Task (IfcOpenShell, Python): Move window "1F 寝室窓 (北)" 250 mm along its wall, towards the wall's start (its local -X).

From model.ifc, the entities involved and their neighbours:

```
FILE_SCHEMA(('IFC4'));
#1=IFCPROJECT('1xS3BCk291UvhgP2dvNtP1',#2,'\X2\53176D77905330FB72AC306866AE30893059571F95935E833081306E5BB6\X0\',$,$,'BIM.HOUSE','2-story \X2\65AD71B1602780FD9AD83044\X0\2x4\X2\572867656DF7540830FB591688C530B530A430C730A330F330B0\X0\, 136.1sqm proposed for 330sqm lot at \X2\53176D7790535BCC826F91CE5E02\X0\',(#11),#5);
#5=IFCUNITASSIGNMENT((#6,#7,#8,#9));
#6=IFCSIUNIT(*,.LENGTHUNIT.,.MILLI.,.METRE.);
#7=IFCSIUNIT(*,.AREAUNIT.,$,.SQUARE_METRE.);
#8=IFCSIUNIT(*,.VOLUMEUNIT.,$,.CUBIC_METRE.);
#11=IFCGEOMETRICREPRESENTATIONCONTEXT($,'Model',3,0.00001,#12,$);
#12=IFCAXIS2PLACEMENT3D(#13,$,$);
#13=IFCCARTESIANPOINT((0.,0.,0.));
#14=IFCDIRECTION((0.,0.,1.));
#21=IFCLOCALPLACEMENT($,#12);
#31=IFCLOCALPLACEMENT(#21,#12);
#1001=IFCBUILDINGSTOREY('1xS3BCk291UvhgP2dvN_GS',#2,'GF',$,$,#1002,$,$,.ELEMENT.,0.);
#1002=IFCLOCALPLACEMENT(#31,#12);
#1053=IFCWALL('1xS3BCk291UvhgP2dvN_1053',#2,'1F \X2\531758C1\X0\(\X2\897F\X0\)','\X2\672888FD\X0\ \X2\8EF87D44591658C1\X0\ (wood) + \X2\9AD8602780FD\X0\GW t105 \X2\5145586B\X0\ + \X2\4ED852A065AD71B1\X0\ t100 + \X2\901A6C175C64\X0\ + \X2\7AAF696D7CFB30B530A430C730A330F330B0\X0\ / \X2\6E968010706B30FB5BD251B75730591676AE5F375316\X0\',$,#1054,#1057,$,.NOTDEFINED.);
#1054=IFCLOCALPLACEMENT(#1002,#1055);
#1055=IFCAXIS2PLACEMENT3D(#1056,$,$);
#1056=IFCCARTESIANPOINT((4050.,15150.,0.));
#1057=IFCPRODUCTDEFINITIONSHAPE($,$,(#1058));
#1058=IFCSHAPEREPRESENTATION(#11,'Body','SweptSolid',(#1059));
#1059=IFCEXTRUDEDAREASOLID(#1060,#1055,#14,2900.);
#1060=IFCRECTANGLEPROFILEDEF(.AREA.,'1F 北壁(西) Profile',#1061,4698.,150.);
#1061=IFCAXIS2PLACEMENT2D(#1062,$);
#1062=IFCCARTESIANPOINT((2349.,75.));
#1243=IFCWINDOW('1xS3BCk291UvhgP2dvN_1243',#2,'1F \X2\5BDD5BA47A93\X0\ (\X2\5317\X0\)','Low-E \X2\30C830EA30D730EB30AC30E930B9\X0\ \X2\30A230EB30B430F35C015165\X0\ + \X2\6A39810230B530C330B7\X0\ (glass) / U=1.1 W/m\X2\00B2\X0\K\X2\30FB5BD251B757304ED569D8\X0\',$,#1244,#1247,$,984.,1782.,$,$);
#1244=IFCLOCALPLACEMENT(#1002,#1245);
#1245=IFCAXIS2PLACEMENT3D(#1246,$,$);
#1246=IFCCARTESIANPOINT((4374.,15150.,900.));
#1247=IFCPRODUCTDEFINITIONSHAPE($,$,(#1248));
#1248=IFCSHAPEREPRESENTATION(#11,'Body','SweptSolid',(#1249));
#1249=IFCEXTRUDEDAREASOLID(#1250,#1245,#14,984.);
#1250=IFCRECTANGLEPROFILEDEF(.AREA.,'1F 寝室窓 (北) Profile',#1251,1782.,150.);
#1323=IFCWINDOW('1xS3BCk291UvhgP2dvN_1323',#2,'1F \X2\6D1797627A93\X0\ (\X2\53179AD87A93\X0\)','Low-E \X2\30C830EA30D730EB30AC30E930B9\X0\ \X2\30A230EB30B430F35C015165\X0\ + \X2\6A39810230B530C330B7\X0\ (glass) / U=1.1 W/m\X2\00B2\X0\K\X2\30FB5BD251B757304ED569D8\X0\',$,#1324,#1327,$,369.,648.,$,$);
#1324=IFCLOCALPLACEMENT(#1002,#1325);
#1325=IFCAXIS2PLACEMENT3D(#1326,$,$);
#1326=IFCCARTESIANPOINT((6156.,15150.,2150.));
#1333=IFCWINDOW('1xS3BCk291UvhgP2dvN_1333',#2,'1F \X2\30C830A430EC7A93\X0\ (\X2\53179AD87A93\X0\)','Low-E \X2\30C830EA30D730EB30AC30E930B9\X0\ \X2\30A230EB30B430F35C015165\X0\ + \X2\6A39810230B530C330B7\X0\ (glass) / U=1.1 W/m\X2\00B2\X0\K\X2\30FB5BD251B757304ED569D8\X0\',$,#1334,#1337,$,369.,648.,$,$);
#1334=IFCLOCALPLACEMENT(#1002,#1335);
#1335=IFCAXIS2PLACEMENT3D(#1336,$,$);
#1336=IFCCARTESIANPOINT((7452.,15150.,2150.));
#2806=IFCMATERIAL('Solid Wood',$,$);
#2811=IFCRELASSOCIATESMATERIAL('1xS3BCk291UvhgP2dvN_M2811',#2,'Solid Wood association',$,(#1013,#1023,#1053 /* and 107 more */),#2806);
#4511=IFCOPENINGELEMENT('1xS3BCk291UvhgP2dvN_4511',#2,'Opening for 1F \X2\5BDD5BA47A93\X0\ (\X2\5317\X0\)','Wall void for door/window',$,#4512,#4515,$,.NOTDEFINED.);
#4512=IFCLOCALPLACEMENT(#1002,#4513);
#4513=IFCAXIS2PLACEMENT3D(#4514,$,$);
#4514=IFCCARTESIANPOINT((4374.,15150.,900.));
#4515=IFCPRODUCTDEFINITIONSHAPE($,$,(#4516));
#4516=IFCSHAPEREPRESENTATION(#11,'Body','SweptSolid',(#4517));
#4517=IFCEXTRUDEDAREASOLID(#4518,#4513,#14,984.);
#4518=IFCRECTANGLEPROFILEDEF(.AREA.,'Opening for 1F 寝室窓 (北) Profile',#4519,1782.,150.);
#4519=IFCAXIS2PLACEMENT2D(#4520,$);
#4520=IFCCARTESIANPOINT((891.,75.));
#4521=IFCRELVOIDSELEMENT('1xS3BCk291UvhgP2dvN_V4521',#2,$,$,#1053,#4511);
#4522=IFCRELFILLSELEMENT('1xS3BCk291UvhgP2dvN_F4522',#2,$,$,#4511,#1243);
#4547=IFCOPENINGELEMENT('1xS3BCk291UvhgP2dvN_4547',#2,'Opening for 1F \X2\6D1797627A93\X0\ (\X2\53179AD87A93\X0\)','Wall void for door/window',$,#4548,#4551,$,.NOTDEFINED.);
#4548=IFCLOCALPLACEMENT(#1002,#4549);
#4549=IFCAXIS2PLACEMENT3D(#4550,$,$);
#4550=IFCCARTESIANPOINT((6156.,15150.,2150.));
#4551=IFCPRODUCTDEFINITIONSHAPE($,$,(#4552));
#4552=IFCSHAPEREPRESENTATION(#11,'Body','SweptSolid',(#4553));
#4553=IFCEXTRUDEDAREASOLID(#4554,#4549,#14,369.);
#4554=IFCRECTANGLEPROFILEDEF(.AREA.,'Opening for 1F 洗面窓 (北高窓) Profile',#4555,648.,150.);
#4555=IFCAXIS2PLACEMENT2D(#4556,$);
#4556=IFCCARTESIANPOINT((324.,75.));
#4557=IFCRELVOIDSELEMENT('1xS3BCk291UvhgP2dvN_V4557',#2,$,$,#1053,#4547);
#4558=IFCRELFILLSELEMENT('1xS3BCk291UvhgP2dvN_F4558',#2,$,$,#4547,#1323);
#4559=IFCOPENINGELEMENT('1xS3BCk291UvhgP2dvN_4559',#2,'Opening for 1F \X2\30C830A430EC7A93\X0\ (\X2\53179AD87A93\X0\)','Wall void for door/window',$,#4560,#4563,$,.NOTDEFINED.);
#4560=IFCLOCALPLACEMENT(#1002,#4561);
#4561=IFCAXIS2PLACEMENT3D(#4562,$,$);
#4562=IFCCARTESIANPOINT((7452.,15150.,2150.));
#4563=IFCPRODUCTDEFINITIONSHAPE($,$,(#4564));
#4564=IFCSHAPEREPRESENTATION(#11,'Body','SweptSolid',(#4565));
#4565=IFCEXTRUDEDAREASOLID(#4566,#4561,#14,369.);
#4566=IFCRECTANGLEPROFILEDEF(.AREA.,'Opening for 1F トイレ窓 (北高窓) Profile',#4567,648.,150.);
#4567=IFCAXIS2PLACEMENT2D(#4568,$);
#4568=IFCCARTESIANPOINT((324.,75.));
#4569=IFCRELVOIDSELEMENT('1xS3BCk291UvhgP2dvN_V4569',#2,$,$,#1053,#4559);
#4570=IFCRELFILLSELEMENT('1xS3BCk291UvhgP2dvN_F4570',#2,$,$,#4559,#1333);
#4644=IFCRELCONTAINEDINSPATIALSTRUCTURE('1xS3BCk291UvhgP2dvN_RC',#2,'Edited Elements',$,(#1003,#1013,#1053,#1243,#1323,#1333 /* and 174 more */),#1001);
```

```python
import ifcopenshell
import ifcopenshell.api.geometry
import ifcopenshell.util.placement
import ifcopenshell.util.unit

model = ifcopenshell.open("model.ifc")
unit_scale = ifcopenshell.util.unit.calculate_unit_scale(model)

window = model.by_id(1243)
opening = window.FillsVoids[0].RelatingOpeningElement
wall = opening.VoidsElements[0].RelatingBuildingElement

wall_matrix = ifcopenshell.util.placement.get_local_placement(wall.ObjectPlacement)
shift = wall_matrix[:3, 0] * -0.25 / unit_scale
before = ifcopenshell.util.placement.get_local_placement(window.ObjectPlacement)[:3, 3].copy()

# The window is not placed relative to its opening, so move both.
for product in (opening, window):
    matrix = ifcopenshell.util.placement.get_local_placement(product.ObjectPlacement)
    matrix[:3, 3] += shift
    ifcopenshell.api.geometry.edit_object_placement(model, product=product, matrix=matrix, is_si=False)

after = ifcopenshell.util.placement.get_local_placement(window.ObjectPlacement)[:3, 3]
print("window moved by", (after - before).round(3) + 0.0)

model.write("model_rev.ifc")
```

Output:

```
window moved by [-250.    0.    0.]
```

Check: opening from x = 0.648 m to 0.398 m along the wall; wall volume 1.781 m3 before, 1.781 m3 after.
